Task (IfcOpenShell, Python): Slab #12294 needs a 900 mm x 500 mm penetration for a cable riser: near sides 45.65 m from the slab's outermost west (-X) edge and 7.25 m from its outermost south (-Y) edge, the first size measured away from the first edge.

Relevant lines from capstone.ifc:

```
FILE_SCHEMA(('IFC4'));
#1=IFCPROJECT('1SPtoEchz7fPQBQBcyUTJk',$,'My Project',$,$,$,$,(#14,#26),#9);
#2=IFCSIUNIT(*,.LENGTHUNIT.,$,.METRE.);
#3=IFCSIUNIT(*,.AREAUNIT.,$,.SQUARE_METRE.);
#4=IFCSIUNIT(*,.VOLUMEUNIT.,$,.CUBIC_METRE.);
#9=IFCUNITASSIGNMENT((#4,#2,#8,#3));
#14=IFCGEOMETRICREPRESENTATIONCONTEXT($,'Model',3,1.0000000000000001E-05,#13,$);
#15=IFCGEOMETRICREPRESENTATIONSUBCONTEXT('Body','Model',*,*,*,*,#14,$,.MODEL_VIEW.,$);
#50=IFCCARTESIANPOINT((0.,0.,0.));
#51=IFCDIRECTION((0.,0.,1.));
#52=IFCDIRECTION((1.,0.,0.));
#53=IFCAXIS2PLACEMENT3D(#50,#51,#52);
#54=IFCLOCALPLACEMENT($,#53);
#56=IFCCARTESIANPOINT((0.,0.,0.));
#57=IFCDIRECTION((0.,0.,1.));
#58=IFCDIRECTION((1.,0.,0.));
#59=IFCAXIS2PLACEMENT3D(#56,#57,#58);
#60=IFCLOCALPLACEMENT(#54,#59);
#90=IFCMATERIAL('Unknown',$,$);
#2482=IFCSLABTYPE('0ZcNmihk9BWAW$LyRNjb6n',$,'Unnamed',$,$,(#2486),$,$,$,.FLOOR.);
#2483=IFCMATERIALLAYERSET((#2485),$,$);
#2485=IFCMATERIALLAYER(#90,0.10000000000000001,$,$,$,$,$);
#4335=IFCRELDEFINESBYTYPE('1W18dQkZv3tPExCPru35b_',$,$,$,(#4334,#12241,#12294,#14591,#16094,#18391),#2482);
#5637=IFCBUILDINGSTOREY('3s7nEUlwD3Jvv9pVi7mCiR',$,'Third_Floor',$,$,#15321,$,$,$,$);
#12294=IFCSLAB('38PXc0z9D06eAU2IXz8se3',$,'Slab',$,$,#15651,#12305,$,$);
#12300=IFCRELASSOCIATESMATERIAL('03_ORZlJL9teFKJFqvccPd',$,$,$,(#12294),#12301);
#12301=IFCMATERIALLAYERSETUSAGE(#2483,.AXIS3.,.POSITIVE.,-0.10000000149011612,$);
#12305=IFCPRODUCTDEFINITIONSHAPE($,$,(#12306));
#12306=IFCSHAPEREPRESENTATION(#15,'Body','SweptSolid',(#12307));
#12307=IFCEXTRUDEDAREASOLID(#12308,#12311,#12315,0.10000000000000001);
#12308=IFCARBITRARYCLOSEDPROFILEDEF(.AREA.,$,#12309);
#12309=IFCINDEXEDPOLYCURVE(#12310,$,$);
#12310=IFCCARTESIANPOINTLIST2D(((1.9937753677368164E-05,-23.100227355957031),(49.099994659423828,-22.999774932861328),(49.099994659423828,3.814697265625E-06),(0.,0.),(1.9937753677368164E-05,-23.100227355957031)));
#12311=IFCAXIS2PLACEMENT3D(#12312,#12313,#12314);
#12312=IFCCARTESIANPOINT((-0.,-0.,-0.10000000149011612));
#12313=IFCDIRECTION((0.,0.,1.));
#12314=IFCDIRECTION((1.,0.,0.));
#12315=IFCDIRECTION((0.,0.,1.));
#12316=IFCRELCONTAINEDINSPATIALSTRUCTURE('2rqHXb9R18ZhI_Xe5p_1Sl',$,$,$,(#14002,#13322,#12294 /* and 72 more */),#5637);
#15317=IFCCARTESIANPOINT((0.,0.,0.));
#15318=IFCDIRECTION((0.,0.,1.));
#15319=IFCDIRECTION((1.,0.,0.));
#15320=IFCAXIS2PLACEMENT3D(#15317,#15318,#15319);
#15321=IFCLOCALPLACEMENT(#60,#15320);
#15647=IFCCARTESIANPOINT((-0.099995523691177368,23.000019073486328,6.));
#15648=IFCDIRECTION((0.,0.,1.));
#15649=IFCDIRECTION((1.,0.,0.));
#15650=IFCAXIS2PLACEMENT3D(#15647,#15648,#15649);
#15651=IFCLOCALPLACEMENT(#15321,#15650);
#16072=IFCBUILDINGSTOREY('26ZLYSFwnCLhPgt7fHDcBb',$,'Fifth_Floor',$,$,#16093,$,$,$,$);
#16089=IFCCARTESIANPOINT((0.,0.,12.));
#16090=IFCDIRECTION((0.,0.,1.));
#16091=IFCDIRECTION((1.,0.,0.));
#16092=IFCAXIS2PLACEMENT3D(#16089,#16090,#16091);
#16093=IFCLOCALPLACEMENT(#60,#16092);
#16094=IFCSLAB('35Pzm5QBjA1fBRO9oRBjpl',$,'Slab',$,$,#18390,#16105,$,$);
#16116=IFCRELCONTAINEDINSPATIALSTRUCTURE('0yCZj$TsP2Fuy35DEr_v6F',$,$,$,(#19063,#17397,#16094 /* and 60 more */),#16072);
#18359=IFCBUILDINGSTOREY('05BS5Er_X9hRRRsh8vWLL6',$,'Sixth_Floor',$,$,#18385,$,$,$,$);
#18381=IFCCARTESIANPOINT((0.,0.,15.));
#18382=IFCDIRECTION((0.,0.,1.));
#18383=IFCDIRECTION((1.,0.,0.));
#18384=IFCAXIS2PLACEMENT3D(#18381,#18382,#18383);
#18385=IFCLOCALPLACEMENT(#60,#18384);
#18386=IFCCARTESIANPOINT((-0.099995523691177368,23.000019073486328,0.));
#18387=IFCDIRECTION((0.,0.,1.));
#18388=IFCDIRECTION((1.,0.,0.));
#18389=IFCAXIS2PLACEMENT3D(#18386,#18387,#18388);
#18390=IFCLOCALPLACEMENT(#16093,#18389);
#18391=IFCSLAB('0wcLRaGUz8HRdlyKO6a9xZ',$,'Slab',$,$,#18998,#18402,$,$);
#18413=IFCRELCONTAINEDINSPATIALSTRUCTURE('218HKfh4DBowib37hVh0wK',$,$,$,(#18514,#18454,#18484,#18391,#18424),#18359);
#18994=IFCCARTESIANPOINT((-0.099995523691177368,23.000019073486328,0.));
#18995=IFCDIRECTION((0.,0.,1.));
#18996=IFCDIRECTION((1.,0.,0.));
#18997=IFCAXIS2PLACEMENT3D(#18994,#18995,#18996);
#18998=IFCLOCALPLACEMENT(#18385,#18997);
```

```python
import numpy as np
import ifcopenshell
import ifcopenshell.api.feature
import ifcopenshell.api.geometry
import ifcopenshell.api.root
import ifcopenshell.geom
import ifcopenshell.util.placement
import ifcopenshell.util.representation
import ifcopenshell.util.shape
import ifcopenshell.util.unit

model = ifcopenshell.open("capstone.ifc")
unit_scale = ifcopenshell.util.unit.calculate_unit_scale(model)
settings = ifcopenshell.geom.settings()


def volume(element):
    """Net volume in cubic metres, openings subtracted."""
    shape = ifcopenshell.geom.create_shape(settings, element)
    return ifcopenshell.util.shape.get_volume(shape.geometry)


slab = model.by_guid("38PXc0z9D06eAU2IXz8se3")
before = volume(slab)

# Extent in the slab's own axes, in metres. The edges named are its -X and -Y sides.
slab_shape = ifcopenshell.geom.create_shape(settings, slab)
vertices = ifcopenshell.util.shape.get_vertices(slab_shape.geometry)
x_min, y_min, bottom = vertices.min(axis=0)
top = vertices[:, 2].max()

opening = ifcopenshell.api.root.create_entity(model, ifc_class="IfcOpeningElement", name="Cable riser opening", predefined_type="OPENING")
context = ifcopenshell.util.representation.get_context(model, "Model", "Body", "MODEL_VIEW")
width, depth = 0.9, 0.5
outline = [(0.0, 0.0), (width, 0.0), (width, depth), (0.0, depth), (0.0, 0.0)]
# Overshoot both faces by 50 mm so the cut is clean.
shape = ifcopenshell.api.geometry.add_slab_representation(
    model, context=context, depth=top - bottom + 0.1, polyline=outline
)
ifcopenshell.api.geometry.assign_representation(model, product=opening, representation=shape)

matrix = ifcopenshell.util.placement.get_local_placement(slab.ObjectPlacement)
matrix[:, 3] = matrix @ np.append(np.array([x_min + 45.65, y_min + 7.25, bottom - 0.05]) / unit_scale, 1.0)
ifcopenshell.api.geometry.edit_object_placement(model, product=opening, matrix=matrix, is_si=False)
ifcopenshell.api.feature.add_feature(model, feature=opening, element=slab)

after = volume(slab)

print(f"slab volume {before:.3f} -> {after:.3f} m3")

model.write("capstone_edited.ifc")
```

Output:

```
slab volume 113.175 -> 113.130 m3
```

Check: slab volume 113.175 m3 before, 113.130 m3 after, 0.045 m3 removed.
